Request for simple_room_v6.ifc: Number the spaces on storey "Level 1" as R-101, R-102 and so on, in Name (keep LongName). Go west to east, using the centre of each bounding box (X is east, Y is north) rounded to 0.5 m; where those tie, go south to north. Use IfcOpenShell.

First a look at what the model holds.

```python
import ifcopenshell
import ifcopenshell.util.element
import ifcopenshell.util.placement

model = ifcopenshell.open("simple_room_v6.ifc")
print(model.schema)
storey = next(s for s in model.by_type("IfcBuildingStorey") if s.Name == "Level 1")
spaces = [e for e in ifcopenshell.util.element.get_decomposition(storey) if e.is_a("IfcSpace")]
for e in sorted(spaces, key=lambda e: e.id()):
    origin = ifcopenshell.util.placement.get_local_placement(e.ObjectPlacement)[:3, 3]
    print(e.id(), e.Name, e.LongName, origin.round(2) + 0.0, sep=" | ")
```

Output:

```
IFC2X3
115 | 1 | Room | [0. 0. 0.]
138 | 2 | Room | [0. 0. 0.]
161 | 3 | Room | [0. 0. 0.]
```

```python
import ifcopenshell
import ifcopenshell.geom
import ifcopenshell.util.element
import ifcopenshell.util.shape

model = ifcopenshell.open("simple_room_v6.ifc")
settings = ifcopenshell.geom.settings()
settings.set("use-world-coords", True)


def centre(element):
    shape = ifcopenshell.geom.create_shape(settings, element)
    return ifcopenshell.util.shape.get_bbox_centroid(shape.geometry)


storey = next(s for s in model.by_type("IfcBuildingStorey") if s.Name == "Level 1")
spaces = [e for e in ifcopenshell.util.element.get_decomposition(storey) if e.is_a("IfcSpace")]

# Insertion points can sit at a corner or the storey origin, so sort by the geometry (in metres).
centres = {e: centre(e) for e in spaces}
spaces.sort(key=lambda e: (round(centres[e][0] / 0.5), centres[e][1]))

for i, e in enumerate(spaces, start=1):
    number = f"R-1{i:02d}"
    e.Name = number
    print(e.id(), number)

model.write("simple_room_v6_updated.ifc")
```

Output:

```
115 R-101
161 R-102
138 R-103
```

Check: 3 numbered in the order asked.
